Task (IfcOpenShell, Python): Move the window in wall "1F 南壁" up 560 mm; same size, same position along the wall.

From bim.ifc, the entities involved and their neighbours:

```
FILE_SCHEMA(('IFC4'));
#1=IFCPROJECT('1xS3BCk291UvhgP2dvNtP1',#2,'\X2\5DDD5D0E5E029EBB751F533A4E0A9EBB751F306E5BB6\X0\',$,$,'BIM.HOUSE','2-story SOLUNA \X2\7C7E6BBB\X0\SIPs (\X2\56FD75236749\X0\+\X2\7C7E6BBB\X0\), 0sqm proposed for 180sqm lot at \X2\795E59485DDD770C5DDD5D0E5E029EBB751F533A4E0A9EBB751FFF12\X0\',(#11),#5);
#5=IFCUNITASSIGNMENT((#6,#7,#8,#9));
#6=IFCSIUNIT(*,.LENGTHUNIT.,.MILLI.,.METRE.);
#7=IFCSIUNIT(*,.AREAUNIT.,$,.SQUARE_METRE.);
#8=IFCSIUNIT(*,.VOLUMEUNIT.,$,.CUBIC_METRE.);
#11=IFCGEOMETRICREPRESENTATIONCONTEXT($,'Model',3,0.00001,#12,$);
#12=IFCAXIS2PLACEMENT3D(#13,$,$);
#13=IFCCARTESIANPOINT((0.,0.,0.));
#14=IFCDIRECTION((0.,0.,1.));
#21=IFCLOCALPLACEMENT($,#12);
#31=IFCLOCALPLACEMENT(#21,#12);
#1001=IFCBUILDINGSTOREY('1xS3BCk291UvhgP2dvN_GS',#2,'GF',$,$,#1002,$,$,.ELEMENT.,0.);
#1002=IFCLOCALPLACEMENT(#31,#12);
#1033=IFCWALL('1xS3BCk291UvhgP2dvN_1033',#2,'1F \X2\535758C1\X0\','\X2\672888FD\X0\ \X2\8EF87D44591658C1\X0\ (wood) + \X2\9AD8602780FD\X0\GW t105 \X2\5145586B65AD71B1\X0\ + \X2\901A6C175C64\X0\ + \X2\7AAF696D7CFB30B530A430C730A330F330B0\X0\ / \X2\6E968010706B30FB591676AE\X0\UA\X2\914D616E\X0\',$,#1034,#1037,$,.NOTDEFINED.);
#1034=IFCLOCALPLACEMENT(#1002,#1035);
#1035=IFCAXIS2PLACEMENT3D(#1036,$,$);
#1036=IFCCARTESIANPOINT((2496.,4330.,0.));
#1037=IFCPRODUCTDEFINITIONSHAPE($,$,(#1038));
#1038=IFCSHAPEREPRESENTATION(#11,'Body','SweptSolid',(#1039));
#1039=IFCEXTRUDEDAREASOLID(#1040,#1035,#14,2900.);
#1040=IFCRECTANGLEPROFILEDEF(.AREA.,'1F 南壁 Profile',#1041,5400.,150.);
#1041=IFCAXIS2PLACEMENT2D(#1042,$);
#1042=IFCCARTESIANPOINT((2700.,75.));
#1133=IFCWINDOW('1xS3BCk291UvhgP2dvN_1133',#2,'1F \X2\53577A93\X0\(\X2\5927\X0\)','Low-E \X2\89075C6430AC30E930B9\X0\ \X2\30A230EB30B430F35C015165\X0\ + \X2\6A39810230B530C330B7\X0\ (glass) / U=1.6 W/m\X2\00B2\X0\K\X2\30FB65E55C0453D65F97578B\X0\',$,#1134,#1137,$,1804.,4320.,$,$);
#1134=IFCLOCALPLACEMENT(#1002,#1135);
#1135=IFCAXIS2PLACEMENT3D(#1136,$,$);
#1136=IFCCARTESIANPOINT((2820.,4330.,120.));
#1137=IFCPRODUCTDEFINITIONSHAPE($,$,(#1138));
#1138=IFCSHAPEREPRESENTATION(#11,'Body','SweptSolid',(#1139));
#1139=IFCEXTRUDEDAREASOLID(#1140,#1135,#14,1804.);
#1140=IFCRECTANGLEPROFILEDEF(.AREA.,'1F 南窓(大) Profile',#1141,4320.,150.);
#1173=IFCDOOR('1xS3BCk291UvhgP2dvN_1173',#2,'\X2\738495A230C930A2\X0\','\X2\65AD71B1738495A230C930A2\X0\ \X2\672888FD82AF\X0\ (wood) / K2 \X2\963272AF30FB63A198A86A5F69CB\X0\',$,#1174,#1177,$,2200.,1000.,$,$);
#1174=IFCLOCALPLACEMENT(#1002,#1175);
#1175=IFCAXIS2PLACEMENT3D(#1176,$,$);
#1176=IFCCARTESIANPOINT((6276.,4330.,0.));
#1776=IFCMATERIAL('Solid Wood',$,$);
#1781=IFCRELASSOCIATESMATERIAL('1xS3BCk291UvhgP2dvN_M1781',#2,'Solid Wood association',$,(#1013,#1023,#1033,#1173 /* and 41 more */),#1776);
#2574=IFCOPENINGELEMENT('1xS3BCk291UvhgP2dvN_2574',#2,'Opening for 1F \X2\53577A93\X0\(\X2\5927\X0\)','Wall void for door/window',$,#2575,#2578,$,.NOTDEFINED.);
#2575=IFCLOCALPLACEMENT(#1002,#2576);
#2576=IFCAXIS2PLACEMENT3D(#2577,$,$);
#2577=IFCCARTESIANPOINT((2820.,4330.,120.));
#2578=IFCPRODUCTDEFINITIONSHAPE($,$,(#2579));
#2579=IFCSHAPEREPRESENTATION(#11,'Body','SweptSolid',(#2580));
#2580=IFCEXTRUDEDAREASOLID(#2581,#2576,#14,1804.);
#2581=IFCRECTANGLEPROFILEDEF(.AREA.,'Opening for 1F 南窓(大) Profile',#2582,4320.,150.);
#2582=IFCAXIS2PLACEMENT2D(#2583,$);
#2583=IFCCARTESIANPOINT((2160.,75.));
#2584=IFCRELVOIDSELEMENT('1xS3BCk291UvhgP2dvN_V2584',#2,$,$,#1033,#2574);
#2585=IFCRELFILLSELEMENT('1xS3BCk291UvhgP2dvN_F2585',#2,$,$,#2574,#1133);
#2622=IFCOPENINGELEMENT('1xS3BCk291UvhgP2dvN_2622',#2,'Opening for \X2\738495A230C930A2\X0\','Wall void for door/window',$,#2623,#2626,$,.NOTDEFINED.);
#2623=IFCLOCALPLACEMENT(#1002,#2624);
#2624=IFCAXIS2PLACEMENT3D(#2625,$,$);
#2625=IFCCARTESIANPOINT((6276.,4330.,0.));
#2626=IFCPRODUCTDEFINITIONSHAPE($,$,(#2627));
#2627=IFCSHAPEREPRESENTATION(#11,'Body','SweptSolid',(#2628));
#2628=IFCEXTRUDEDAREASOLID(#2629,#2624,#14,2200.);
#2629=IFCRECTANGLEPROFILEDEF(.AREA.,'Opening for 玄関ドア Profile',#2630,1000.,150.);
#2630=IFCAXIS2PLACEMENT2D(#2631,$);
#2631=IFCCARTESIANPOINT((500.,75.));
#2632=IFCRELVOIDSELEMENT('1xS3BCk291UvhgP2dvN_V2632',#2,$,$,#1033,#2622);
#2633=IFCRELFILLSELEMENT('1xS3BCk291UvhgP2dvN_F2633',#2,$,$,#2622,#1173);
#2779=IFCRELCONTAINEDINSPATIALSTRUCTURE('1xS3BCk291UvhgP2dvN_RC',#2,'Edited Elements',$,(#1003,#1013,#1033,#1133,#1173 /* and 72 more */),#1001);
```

```python
import numpy as np
import ifcopenshell
import ifcopenshell.api.geometry
import ifcopenshell.util.placement
import ifcopenshell.util.unit

model = ifcopenshell.open("bim.ifc")
unit_scale = ifcopenshell.util.unit.calculate_unit_scale(model)

window = model.by_id(1133)
opening = window.FillsVoids[0].RelatingOpeningElement
dz = 0.56 / unit_scale

shift = np.array([0.0, 0.0, dz])
# The window is not placed relative to its opening, so move both.
for product in (opening, window):
    matrix = ifcopenshell.util.placement.get_local_placement(product.ObjectPlacement)
    matrix[:3, 3] += shift
    ifcopenshell.api.geometry.edit_object_placement(model, product=product, matrix=matrix, is_si=False)

print(f"moved by {dz * unit_scale:+.3f} m")

model.write("bim_edited.ifc")
```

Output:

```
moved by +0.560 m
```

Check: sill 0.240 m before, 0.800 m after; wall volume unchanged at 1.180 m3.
